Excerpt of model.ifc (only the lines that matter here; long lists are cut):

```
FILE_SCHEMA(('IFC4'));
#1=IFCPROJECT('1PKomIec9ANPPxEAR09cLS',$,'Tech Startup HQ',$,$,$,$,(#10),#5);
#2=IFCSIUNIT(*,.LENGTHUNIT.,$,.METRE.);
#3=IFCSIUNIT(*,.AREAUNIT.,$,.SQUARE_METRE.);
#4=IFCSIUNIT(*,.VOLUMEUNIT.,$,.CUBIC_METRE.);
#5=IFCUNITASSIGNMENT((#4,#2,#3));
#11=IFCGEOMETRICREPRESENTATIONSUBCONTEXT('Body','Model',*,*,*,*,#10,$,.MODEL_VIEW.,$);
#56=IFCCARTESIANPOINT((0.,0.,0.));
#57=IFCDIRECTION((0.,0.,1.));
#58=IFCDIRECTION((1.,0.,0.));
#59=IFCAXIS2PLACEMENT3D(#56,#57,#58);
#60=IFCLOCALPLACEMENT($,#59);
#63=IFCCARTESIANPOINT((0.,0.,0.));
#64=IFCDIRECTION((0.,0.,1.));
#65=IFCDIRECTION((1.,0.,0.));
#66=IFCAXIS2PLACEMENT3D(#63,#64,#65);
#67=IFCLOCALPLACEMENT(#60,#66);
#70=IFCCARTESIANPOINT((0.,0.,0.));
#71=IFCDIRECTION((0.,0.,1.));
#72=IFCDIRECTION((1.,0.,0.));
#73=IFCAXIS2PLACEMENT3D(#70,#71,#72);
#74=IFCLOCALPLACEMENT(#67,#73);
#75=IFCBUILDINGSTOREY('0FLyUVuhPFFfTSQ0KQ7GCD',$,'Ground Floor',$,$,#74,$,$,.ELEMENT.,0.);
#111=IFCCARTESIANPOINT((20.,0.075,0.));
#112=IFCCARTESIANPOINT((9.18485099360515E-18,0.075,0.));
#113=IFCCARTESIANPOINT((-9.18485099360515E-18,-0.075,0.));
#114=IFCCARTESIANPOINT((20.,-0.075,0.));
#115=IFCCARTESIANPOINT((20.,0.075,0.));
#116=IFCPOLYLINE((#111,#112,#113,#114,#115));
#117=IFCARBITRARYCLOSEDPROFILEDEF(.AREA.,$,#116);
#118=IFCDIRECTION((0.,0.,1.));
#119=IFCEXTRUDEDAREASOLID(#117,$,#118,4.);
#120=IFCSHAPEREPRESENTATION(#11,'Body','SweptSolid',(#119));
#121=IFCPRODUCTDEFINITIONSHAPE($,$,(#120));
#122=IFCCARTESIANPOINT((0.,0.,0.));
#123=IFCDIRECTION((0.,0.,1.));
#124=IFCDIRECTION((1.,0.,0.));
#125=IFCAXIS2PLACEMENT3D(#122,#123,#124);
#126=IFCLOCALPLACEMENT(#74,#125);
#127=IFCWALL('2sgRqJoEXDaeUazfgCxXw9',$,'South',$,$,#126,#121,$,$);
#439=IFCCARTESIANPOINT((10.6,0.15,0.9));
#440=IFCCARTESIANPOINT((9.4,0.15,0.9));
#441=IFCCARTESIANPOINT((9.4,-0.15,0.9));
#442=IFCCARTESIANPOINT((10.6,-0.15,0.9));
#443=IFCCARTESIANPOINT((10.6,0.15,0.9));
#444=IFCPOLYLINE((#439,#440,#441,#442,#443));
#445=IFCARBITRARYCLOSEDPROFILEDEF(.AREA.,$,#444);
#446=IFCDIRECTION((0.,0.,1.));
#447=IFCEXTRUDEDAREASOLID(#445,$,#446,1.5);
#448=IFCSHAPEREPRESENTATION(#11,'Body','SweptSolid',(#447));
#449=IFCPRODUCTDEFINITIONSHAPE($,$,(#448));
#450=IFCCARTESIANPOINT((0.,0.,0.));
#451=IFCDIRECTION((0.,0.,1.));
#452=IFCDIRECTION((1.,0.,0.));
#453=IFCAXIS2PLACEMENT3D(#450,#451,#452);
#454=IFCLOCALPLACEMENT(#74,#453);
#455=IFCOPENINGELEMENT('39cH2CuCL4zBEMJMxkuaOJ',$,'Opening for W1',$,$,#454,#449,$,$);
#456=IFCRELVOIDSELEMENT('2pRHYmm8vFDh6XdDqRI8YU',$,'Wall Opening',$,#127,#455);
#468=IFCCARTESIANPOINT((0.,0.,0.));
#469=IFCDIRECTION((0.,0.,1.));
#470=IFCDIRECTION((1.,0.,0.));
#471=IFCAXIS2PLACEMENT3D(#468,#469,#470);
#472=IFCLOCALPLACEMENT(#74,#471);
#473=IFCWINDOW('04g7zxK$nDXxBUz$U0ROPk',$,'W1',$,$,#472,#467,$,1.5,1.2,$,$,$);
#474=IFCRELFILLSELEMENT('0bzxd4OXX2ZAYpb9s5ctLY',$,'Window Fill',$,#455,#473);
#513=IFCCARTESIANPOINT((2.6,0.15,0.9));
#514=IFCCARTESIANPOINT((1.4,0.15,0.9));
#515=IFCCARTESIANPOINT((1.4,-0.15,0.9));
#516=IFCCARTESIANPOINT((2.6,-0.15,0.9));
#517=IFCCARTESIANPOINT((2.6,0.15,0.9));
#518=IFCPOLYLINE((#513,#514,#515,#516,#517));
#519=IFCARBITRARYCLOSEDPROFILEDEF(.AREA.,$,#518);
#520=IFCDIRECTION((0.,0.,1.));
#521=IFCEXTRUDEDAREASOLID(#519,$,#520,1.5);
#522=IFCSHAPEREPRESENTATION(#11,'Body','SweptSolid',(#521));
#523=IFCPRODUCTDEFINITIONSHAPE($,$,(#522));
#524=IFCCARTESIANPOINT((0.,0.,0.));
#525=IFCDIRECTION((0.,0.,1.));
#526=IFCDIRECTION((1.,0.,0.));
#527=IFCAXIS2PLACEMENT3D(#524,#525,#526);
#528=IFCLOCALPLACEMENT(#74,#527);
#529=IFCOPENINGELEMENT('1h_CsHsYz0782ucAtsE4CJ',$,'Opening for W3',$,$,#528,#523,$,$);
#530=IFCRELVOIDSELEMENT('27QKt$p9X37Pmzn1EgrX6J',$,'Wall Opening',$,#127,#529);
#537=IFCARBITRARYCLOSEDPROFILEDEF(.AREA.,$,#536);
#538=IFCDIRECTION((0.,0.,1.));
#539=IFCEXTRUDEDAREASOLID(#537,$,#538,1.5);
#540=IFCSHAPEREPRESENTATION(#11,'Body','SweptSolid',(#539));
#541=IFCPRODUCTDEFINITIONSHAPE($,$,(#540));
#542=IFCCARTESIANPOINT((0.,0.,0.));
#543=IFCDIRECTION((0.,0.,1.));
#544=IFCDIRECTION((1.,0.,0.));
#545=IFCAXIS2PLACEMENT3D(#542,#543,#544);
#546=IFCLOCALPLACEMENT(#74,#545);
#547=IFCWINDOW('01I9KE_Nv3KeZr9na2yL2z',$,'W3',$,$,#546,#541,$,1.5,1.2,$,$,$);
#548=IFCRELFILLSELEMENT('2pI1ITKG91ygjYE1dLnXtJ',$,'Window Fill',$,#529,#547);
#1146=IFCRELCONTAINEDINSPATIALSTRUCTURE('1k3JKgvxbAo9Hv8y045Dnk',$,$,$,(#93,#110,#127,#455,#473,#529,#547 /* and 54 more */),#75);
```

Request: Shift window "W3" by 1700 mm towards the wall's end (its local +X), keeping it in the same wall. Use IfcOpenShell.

```python
import ifcopenshell
import ifcopenshell.api.geometry
import ifcopenshell.util.placement
import ifcopenshell.util.unit

model = ifcopenshell.open("model.ifc")
unit_scale = ifcopenshell.util.unit.calculate_unit_scale(model)

window = model.by_guid("01I9KE_Nv3KeZr9na2yL2z")
opening = window.FillsVoids[0].RelatingOpeningElement
wall = opening.VoidsElements[0].RelatingBuildingElement

wall_matrix = ifcopenshell.util.placement.get_local_placement(wall.ObjectPlacement)
shift = wall_matrix[:3, 0] * 1.7 / unit_scale
before = ifcopenshell.util.placement.get_local_placement(window.ObjectPlacement)[:3, 3].copy()

# The window is not placed relative to its opening, so move both.
for product in (opening, window):
    matrix = ifcopenshell.util.placement.get_local_placement(product.ObjectPlacement)
    matrix[:3, 3] += shift
    ifcopenshell.api.geometry.edit_object_placement(model, product=product, matrix=matrix, is_si=False)

after = ifcopenshell.util.placement.get_local_placement(window.ObjectPlacement)[:3, 3]
print("window moved by", (after - before).round(3) + 0.0)

model.write("model_updated.ifc")
```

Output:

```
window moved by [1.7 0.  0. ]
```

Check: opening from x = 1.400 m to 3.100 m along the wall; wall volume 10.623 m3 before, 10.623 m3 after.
